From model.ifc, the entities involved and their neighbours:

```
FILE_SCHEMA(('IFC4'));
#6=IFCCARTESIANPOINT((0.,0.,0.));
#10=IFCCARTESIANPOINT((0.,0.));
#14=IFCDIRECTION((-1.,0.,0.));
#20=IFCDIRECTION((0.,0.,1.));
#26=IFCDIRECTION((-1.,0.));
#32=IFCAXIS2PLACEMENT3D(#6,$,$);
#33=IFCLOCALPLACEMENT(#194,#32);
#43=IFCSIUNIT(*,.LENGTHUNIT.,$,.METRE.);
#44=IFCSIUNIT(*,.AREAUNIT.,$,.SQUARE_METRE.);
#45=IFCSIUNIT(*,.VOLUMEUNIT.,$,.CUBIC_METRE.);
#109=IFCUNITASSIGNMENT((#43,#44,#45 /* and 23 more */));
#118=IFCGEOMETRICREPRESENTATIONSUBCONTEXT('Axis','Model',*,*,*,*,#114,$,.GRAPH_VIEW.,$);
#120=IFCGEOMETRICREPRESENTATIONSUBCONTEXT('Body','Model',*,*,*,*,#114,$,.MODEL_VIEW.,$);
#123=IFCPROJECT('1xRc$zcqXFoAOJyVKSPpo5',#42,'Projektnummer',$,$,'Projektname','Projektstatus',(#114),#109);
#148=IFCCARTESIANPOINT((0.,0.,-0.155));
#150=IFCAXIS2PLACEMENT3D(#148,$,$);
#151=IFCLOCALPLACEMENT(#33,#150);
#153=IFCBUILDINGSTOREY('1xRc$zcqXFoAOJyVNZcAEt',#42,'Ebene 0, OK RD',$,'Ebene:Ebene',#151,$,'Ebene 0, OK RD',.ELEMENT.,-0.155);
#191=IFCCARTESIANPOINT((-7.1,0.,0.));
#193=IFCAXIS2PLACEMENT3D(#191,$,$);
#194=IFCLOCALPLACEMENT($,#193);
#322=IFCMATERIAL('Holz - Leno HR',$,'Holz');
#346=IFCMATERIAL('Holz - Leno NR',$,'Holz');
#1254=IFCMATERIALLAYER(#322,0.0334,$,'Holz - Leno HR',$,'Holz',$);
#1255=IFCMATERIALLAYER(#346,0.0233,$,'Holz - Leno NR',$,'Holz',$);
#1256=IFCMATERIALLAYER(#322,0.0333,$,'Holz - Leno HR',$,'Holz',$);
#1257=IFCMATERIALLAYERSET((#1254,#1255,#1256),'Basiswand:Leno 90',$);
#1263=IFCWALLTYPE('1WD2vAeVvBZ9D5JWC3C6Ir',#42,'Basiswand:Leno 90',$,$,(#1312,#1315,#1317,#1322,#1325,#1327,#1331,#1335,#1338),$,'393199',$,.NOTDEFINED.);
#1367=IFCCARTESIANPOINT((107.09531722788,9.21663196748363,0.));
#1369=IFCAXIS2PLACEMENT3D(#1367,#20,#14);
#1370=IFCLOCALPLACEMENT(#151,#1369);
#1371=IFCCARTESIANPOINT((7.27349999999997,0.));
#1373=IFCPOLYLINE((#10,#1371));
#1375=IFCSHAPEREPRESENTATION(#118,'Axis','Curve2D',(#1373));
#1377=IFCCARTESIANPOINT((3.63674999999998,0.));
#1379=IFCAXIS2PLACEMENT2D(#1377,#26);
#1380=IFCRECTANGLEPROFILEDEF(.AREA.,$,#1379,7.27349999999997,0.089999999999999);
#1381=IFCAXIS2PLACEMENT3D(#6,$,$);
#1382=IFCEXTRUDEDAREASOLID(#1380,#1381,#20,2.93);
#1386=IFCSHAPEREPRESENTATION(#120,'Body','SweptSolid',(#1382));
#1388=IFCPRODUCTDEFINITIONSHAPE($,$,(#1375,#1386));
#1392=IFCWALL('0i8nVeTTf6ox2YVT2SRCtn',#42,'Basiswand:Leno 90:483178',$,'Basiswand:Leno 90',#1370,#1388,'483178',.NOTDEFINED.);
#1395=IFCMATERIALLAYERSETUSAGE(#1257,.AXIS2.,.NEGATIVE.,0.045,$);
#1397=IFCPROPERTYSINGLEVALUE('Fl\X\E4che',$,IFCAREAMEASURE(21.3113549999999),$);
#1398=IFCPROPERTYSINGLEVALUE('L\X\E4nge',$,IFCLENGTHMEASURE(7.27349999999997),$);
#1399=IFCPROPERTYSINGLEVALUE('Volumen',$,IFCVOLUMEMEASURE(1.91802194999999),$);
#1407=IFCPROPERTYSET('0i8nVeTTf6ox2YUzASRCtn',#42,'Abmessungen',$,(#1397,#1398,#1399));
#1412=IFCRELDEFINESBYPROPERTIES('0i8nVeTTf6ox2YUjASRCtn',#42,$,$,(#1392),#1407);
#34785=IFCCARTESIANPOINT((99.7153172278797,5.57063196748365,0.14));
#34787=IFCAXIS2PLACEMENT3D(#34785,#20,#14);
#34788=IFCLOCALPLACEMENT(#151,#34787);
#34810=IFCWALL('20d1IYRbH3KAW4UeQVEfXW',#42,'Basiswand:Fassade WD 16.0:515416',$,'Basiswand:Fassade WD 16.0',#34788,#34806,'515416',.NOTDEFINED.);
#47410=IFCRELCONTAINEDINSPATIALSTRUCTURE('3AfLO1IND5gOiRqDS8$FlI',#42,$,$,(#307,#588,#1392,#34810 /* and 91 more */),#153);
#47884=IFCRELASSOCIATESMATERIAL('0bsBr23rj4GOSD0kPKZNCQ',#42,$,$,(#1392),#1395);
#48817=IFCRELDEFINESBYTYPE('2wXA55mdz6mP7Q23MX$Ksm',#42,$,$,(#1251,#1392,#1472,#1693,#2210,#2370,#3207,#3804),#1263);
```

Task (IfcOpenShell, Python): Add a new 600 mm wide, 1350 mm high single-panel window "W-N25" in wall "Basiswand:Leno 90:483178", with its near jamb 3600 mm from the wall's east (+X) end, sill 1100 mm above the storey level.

```python
import numpy as np
import ifcopenshell
import ifcopenshell.api.feature
import ifcopenshell.api.geometry
import ifcopenshell.api.pset
import ifcopenshell.api.root
import ifcopenshell.api.spatial
import ifcopenshell.geom
import ifcopenshell.util.element
import ifcopenshell.util.placement
import ifcopenshell.util.representation
import ifcopenshell.util.shape
import ifcopenshell.util.unit

model = ifcopenshell.open("model.ifc")
unit_scale = ifcopenshell.util.unit.calculate_unit_scale(model)
area_scale = ifcopenshell.util.unit.calculate_unit_scale(model, "AREAUNIT")
volume_scale = ifcopenshell.util.unit.calculate_unit_scale(model, "VOLUMEUNIT")
settings = ifcopenshell.geom.settings()


def volume(element):
    """Net volume in cubic metres, openings subtracted."""
    shape = ifcopenshell.geom.create_shape(settings, element)
    return ifcopenshell.util.shape.get_volume(shape.geometry)


wall = model.by_guid("0i8nVeTTf6ox2YVT2SRCtn")
storey = ifcopenshell.util.element.get_container(wall, ifc_class="IfcBuildingStorey")
context = ifcopenshell.util.representation.get_context(model, "Model", "Body", "MODEL_VIEW")
before = volume(wall)

width, height, from_end, sill = 0.6, 1.35, 3.6, 1.1  # metres

# The wall runs along its own X axis, and the end named is its -X end.
wall_shape = ifcopenshell.geom.create_shape(settings, wall)
x, y, z = ifcopenshell.util.shape.get_vertices(wall_shape.geometry).T
start = x.min() + from_end
face, thickness = float(y.min()), float(y.max() - y.min())
wall_matrix = ifcopenshell.util.placement.get_local_placement(wall.ObjectPlacement)
level = ifcopenshell.util.placement.get_local_placement(storey.ObjectPlacement)[2, 3]


def in_wall(x, y):
    """Placement at x, y metres in the wall's axes, at sill height."""
    matrix = wall_matrix.copy()
    matrix[:, 3] = wall_matrix @ np.array([x / unit_scale, y / unit_scale, 0.0, 1.0])
    matrix[2, 3] = level + sill / unit_scale
    return matrix


# Opening: a box that overshoots both wall faces by 50 mm.
opening = ifcopenshell.api.root.create_entity(model, ifc_class="IfcOpeningElement", predefined_type="OPENING")
box = ifcopenshell.api.geometry.add_wall_representation(
    model, context=context, length=width, height=height, thickness=thickness + 0.1
)
ifcopenshell.api.geometry.assign_representation(model, product=opening, representation=box)
ifcopenshell.api.geometry.edit_object_placement(model, product=opening, matrix=in_wall(start, face - 0.05), is_si=False)
ifcopenshell.api.feature.add_feature(model, feature=opening, element=wall)

window = ifcopenshell.api.root.create_entity(model, ifc_class="IfcWindow", name="W-N25", predefined_type="WINDOW")
window.OverallWidth, window.OverallHeight = width / unit_scale, height / unit_scale
window.PartitioningType = "SINGLE_PANEL"
body = ifcopenshell.api.geometry.add_window_representation(
    model,
    context=context,
    overall_width=window.OverallWidth,
    overall_height=window.OverallHeight,
    partition_type="SINGLE_PANEL",
)
ifcopenshell.api.geometry.assign_representation(model, product=window, representation=body)
ifcopenshell.api.spatial.assign_container(model, products=[window], relating_structure=storey)
ifcopenshell.api.feature.add_filling(model, opening=opening, element=window)

# Centre the window in the wall's thickness.
ifcopenshell.api.geometry.edit_object_placement(model, product=window, matrix=in_wall(start, face), is_si=False)
window_shape = ifcopenshell.geom.create_shape(settings, window)
depth = ifcopenshell.util.shape.get_vertices(window_shape.geometry)[:, 1]
offset = face + thickness / 2 - (depth.min() + depth.max()) / 2
ifcopenshell.api.geometry.edit_object_placement(model, product=window, matrix=in_wall(start, offset), is_si=False)

after = volume(wall)

# Update the wall's stored quantities.
pset = model.by_id(ifcopenshell.util.element.get_pset(wall, "Abmessungen", should_inherit=False)["id"])
ifcopenshell.api.pset.edit_pset(model, pset=pset, properties={
    "Fläche": model.create_entity("IfcAreaMeasure", after / thickness / area_scale),
    "Volumen": model.create_entity("IfcVolumeMeasure", after / volume_scale),
})

print(f"wall volume {before:.3f} -> {after:.3f} m3")

model.write("model_rev.ifc")
```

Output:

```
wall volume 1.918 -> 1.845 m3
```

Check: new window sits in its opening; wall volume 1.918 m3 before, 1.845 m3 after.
